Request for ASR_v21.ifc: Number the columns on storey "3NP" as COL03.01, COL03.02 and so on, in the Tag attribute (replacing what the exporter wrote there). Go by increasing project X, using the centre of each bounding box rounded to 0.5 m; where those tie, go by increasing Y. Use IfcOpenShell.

First a look at what the model holds.

```python
import ifcopenshell
import ifcopenshell.util.element
import ifcopenshell.util.placement

model = ifcopenshell.open("ASR_v21.ifc")
print(model.schema)
storey = next(s for s in model.by_type("IfcBuildingStorey") if s.Name == "3NP")
columns = [e for e in ifcopenshell.util.element.get_decomposition(storey) if e.is_a("IfcColumn")]
for e in sorted(columns, key=lambda e: e.id()):
    origin = ifcopenshell.util.placement.get_local_placement(e.ObjectPlacement)[:3, 3]
    print(e.id(), e.Tag, e.Name, origin.round(2) + 0.0, sep=" | ")
```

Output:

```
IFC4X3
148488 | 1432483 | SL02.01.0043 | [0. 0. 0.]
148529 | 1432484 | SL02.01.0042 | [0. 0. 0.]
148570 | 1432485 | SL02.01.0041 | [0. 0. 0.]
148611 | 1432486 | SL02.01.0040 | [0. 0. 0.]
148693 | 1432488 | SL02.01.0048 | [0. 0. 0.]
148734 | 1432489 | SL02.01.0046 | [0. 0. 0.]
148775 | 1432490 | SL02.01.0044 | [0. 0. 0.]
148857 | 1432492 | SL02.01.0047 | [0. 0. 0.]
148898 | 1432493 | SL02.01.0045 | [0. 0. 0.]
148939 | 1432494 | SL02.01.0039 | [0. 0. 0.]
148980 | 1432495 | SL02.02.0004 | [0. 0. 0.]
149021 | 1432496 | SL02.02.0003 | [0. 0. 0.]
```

```python
import ifcopenshell
import ifcopenshell.geom
import ifcopenshell.util.element
import ifcopenshell.util.shape

model = ifcopenshell.open("ASR_v21.ifc")
settings = ifcopenshell.geom.settings()
settings.set("use-world-coords", True)


def centre(element):
    shape = ifcopenshell.geom.create_shape(settings, element)
    return ifcopenshell.util.shape.get_bbox_centroid(shape.geometry)


storey = next(s for s in model.by_type("IfcBuildingStorey") if s.Name == "3NP")
columns = [e for e in ifcopenshell.util.element.get_decomposition(storey) if e.is_a("IfcColumn")]

# Insertion points can sit at a corner or the storey origin, so sort by the geometry (in metres).
centres = {e: centre(e) for e in columns}
columns.sort(key=lambda e: (round(centres[e][0] / 0.5), centres[e][1]))

for i, e in enumerate(columns, start=1):
    number = f"COL03.{i:02d}"
    e.Tag = number
    print(e.id(), number)

model.write("ASR_v21_updated.ifc")
```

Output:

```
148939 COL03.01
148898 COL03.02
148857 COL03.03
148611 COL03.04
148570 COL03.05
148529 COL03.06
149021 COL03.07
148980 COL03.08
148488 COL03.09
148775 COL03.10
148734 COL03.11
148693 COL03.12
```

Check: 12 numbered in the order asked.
